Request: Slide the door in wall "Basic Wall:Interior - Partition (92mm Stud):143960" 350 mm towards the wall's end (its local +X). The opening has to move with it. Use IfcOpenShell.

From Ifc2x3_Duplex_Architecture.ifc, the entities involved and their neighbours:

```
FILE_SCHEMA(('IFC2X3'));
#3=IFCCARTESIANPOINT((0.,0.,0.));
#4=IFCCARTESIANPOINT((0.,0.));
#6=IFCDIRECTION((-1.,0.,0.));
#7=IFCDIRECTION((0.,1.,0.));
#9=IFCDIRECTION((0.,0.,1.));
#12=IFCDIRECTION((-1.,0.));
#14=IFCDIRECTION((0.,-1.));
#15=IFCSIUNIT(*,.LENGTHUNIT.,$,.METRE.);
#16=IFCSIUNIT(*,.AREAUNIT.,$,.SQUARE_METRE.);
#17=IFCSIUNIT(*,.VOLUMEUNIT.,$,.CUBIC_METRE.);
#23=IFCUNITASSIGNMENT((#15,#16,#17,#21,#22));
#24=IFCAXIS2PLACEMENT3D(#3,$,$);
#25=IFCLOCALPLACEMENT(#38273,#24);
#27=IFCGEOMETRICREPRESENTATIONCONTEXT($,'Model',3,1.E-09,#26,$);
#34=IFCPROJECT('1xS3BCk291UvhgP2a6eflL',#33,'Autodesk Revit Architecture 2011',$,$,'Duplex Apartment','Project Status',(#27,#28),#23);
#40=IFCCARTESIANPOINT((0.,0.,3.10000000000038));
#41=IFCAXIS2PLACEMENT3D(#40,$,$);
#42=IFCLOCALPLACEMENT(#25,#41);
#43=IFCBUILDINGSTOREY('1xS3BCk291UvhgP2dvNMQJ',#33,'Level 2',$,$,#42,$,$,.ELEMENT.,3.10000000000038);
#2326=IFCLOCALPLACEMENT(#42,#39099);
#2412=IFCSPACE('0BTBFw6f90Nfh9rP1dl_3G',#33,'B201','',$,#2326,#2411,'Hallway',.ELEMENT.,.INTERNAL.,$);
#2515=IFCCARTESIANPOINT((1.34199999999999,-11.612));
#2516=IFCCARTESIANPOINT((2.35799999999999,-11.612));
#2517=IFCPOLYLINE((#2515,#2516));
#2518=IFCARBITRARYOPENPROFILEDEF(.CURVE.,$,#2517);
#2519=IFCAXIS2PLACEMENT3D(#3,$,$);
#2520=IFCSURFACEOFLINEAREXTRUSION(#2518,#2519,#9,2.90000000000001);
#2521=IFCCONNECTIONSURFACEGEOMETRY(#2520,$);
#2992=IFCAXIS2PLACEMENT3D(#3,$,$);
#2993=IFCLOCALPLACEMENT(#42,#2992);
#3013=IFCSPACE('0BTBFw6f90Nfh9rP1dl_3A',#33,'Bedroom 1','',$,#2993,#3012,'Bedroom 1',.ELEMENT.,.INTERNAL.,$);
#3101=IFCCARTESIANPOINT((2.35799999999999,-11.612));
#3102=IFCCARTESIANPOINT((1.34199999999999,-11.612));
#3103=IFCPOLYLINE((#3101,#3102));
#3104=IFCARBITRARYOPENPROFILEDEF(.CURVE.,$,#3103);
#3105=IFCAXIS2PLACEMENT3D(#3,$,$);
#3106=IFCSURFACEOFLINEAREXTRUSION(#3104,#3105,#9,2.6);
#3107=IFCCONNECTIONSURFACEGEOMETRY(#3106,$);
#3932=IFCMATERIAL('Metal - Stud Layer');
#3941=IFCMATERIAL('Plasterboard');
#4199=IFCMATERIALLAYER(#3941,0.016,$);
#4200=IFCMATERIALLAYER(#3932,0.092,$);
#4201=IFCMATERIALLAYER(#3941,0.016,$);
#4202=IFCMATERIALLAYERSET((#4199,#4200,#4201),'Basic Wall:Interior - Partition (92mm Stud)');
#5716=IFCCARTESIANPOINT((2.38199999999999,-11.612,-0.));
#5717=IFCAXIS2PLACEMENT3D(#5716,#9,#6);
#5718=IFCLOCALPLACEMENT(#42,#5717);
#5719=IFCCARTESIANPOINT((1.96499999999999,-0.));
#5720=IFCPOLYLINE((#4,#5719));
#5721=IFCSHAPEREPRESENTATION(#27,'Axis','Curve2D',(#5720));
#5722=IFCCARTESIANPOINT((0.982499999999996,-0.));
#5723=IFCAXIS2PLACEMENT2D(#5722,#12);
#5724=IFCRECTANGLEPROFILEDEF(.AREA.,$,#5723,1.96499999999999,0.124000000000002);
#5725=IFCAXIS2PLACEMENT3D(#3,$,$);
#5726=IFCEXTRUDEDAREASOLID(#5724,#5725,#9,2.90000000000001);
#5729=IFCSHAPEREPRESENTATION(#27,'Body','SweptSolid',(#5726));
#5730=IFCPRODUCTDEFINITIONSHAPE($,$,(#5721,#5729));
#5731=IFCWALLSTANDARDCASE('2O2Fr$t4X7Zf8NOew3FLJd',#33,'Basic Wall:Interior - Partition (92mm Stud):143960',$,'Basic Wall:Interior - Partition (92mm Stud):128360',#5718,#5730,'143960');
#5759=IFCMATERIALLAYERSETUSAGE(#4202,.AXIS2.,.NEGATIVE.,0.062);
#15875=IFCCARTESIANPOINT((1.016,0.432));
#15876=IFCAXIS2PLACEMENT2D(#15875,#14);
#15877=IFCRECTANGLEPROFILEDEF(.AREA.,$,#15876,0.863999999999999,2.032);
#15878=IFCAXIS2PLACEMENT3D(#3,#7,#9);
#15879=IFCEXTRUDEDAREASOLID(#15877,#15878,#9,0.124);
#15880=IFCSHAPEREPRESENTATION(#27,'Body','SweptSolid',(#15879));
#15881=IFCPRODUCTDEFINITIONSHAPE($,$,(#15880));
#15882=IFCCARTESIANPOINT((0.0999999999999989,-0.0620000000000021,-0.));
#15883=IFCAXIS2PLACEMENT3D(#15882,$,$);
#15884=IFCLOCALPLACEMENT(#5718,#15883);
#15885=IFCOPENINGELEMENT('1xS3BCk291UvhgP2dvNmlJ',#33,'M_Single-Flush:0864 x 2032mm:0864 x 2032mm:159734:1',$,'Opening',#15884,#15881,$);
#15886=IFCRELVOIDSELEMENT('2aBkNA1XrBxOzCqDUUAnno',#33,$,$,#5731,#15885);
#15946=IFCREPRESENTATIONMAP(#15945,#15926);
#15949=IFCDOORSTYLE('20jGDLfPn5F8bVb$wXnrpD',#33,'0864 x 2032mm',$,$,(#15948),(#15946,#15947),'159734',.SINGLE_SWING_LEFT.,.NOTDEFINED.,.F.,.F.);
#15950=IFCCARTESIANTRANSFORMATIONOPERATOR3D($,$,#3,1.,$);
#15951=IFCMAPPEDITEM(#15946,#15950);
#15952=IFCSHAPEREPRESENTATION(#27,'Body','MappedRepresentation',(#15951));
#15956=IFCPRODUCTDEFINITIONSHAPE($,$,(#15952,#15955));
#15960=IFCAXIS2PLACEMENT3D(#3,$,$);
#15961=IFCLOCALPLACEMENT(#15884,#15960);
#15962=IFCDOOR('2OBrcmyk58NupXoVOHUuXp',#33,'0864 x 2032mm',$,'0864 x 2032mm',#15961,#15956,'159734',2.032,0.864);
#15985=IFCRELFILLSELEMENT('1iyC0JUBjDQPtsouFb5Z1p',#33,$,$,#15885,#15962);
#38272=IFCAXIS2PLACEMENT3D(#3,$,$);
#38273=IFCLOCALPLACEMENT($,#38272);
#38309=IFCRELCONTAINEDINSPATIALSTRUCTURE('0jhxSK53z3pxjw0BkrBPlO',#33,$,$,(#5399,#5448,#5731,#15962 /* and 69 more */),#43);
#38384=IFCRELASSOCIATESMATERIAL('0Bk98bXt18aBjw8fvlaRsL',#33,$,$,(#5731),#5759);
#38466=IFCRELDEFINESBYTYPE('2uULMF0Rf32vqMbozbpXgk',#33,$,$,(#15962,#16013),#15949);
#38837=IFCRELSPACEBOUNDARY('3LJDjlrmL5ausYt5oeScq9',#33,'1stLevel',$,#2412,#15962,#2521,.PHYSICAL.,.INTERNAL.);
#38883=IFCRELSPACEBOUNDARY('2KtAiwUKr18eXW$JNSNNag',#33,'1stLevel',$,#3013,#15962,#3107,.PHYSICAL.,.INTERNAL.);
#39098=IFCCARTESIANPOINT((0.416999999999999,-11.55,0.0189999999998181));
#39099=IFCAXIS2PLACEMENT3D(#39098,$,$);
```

```python
import numpy as np
import ifcopenshell
import ifcopenshell.api.geometry
import ifcopenshell.util.placement
import ifcopenshell.util.unit

model = ifcopenshell.open("Ifc2x3_Duplex_Architecture.ifc")
unit_scale = ifcopenshell.util.unit.calculate_unit_scale(model)

door = model.by_guid("2OBrcmyk58NupXoVOHUuXp")
opening = door.FillsVoids[0].RelatingOpeningElement
wall = opening.VoidsElements[0].RelatingBuildingElement

wall_matrix = ifcopenshell.util.placement.get_local_placement(wall.ObjectPlacement)
shift = wall_matrix[:3, 0] * 0.35 / unit_scale
before = ifcopenshell.util.placement.get_local_placement(door.ObjectPlacement)[:3, 3].copy()

# The door is placed relative to its opening, so it follows when the opening moves.
matrix = ifcopenshell.util.placement.get_local_placement(opening.ObjectPlacement)
matrix[:3, 3] += shift
ifcopenshell.api.geometry.edit_object_placement(
    model, product=opening, matrix=matrix, is_si=False, should_transform_children=True
)

# Space boundary surfaces are stored in each space's coordinates; move them too.
for rel in door.ProvidesBoundaries:
    if not rel.ConnectionGeometry:
        continue
    surface = rel.ConnectionGeometry.SurfaceOnRelatingElement
    space_matrix = ifcopenshell.util.placement.get_local_placement(rel.RelatingSpace.ObjectPlacement)
    point = np.array(surface.Position.Location.Coordinates) + space_matrix[:3, :3].T @ shift
    surface.Position = model.createIfcAxis2Placement3D(
        model.createIfcCartesianPoint(point.tolist()), surface.Position.Axis, surface.Position.RefDirection
    )

after = ifcopenshell.util.placement.get_local_placement(door.ObjectPlacement)[:3, 3]
print("door moved by", (after - before).round(3) + 0.0)

model.write("Ifc2x3_Duplex_Architecture_rev.ifc")
```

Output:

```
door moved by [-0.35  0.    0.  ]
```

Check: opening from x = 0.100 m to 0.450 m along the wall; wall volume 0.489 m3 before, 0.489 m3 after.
